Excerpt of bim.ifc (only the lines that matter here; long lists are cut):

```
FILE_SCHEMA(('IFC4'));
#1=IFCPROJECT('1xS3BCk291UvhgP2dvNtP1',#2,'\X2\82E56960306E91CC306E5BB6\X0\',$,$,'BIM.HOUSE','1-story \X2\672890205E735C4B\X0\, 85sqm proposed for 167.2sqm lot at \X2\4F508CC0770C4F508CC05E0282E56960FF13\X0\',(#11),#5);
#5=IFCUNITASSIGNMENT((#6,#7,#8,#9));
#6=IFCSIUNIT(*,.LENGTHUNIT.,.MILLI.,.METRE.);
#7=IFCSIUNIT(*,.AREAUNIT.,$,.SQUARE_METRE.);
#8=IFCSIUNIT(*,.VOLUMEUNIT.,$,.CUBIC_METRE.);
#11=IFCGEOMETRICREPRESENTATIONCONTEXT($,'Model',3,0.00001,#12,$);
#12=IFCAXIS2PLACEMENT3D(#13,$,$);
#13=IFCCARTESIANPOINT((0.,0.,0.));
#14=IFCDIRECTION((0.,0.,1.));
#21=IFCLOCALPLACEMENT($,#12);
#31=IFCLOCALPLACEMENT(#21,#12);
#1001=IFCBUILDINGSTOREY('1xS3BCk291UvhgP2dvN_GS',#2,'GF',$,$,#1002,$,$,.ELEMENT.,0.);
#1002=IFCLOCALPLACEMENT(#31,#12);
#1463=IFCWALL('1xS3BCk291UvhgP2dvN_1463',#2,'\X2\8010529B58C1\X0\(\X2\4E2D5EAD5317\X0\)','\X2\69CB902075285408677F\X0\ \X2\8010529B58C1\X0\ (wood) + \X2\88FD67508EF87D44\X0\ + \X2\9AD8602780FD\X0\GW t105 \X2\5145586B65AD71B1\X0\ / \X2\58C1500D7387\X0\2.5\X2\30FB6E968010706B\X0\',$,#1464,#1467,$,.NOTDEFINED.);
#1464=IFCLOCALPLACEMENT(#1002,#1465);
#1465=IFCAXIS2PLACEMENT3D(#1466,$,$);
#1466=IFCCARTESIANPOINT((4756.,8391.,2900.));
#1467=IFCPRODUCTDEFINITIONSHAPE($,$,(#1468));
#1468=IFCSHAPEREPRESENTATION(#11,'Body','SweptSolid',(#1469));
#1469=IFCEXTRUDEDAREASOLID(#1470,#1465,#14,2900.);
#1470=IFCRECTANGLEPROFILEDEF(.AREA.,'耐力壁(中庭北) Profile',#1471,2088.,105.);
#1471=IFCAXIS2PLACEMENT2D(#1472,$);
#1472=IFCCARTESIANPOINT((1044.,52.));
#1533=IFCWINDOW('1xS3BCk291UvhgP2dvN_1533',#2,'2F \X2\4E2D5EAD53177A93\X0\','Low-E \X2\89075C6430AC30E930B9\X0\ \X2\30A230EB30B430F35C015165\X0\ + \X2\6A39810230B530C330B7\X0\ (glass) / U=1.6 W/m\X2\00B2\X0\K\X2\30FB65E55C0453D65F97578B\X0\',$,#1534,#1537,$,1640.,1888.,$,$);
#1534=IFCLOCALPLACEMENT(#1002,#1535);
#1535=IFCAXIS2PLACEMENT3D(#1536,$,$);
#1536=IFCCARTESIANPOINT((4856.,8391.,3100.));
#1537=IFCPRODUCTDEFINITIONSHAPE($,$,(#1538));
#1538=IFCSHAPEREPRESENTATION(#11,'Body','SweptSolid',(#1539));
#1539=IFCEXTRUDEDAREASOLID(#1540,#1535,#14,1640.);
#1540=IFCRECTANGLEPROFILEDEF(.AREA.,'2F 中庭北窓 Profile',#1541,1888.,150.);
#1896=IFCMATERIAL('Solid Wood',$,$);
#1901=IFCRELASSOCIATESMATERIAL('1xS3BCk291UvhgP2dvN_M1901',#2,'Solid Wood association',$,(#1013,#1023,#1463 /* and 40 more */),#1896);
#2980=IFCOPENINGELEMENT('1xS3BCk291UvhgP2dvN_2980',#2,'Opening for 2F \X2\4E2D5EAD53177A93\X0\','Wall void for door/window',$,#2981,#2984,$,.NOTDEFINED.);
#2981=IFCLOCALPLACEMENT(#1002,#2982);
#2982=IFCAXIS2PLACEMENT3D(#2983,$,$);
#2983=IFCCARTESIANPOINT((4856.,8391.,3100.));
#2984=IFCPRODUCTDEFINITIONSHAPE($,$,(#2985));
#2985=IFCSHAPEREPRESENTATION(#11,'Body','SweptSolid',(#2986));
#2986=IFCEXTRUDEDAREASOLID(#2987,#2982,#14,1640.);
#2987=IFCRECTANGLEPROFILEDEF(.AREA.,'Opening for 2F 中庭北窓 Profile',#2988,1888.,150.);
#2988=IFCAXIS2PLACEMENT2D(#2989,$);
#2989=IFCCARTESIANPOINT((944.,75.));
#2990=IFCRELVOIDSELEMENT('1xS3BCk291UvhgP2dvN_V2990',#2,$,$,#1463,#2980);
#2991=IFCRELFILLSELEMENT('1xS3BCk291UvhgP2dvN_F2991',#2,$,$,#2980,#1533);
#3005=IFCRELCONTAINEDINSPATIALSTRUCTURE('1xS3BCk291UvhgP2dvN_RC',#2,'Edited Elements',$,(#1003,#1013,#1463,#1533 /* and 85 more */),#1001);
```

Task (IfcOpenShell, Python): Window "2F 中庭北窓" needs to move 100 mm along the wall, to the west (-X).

```python
import ifcopenshell
import ifcopenshell.api.geometry
import ifcopenshell.util.placement
import ifcopenshell.util.unit

model = ifcopenshell.open("bim.ifc")
unit_scale = ifcopenshell.util.unit.calculate_unit_scale(model)

window = model.by_id(1533)
opening = window.FillsVoids[0].RelatingOpeningElement
wall = opening.VoidsElements[0].RelatingBuildingElement

wall_matrix = ifcopenshell.util.placement.get_local_placement(wall.ObjectPlacement)
shift = wall_matrix[:3, 0] * -0.1 / unit_scale
before = ifcopenshell.util.placement.get_local_placement(window.ObjectPlacement)[:3, 3].copy()

# The window is not placed relative to its opening, so move both.
for product in (opening, window):
    matrix = ifcopenshell.util.placement.get_local_placement(product.ObjectPlacement)
    matrix[:3, 3] += shift
    ifcopenshell.api.geometry.edit_object_placement(model, product=product, matrix=matrix, is_si=False)

after = ifcopenshell.util.placement.get_local_placement(window.ObjectPlacement)[:3, 3]
print("window moved by", (after - before).round(3) + 0.0)

model.write("bim_edited.ifc")
```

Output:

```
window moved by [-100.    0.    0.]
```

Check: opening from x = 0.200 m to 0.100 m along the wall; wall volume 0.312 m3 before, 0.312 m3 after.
